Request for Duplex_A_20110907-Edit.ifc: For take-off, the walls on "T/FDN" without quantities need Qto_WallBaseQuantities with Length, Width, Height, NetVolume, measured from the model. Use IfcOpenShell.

First a look at what the model holds.

```python
import ifcopenshell
import ifcopenshell.util.element
import ifcopenshell.util.unit

model = ifcopenshell.open("Duplex_A_20110907-Edit.ifc")
print(model.schema)
for unit_type in ("LENGTHUNIT", "AREAUNIT", "VOLUMEUNIT"):
    print(unit_type, ifcopenshell.util.unit.calculate_unit_scale(model, unit_type))
storey = next(s for s in model.by_type("IfcBuildingStorey") if s.Name == "T/FDN")
walls = [e for e in ifcopenshell.util.element.get_decomposition(storey) if e.is_a("IfcWall")]
for e in sorted(walls, key=lambda e: e.id()):
    print(e.id(), e.is_a(), e.Name, list(ifcopenshell.util.element.get_psets(e, qtos_only=True)), sep=" | ")
```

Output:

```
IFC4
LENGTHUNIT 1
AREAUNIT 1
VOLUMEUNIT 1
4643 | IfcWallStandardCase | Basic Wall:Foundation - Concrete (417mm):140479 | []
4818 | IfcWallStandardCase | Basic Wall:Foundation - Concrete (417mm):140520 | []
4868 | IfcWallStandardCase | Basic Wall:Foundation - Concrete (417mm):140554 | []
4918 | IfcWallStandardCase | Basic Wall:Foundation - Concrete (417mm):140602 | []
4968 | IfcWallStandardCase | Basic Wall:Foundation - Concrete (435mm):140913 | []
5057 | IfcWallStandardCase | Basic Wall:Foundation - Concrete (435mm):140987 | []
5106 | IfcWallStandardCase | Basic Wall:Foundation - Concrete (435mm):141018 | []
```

```python
import ifcopenshell
import ifcopenshell.api.pset
import ifcopenshell.geom
import ifcopenshell.util.element
import ifcopenshell.util.shape
import ifcopenshell.util.unit

model = ifcopenshell.open("Duplex_A_20110907-Edit.ifc")
unit_scale = ifcopenshell.util.unit.calculate_unit_scale(model)
volume_scale = ifcopenshell.util.unit.calculate_unit_scale(model, "VOLUMEUNIT")
settings = ifcopenshell.geom.settings()

storey = next(s for s in model.by_type("IfcBuildingStorey") if s.Name == "T/FDN")
walls = [e for e in ifcopenshell.util.element.get_decomposition(storey) if e.is_a("IfcWall")]

for e in sorted(walls, key=lambda e: e.id()):
    if ifcopenshell.util.element.get_psets(e, qtos_only=True, should_inherit=False):
        continue
    # Geometry comes back in metres, in the element's own axes.
    shape = ifcopenshell.geom.create_shape(settings, e)
    values = {
        "Length": ifcopenshell.util.shape.get_x(shape.geometry) / unit_scale,
        "Width": ifcopenshell.util.shape.get_y(shape.geometry) / unit_scale,
        "Height": ifcopenshell.util.shape.get_z(shape.geometry) / unit_scale,
        "NetVolume": ifcopenshell.util.shape.get_volume(shape.geometry) / volume_scale,
    }
    qto = ifcopenshell.api.pset.add_qto(model, product=e, name="Qto_WallBaseQuantities")
    ifcopenshell.api.pset.edit_qto(model, qto=qto, properties=values)
    print(e.id(), {k: round(v, 3) for k, v in values.items()})

model.write("Duplex_A_20110907-Edit_updated.ifc")
```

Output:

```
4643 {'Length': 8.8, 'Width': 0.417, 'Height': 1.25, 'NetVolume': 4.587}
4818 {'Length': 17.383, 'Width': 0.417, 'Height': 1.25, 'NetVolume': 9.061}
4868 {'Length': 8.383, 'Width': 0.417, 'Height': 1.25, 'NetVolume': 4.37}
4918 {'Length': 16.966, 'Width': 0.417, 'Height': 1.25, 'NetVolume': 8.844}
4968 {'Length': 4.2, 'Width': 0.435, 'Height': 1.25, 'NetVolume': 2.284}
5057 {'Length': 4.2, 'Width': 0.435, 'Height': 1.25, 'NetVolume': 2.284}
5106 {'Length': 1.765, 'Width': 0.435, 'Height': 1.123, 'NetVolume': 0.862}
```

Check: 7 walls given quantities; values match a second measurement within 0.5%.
